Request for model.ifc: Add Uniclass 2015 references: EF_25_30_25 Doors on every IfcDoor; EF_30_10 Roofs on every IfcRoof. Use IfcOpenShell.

First a look at what the model holds.

```python
import ifcopenshell

model = ifcopenshell.open("model.ifc")
print(model.schema)
print("classifications:", [c.Name for c in model.by_type("IfcClassification")])
for ifc_class in ("IfcDoor", "IfcRoof", "IfcStair", "IfcWall", "IfcWindow"):
    print(ifc_class, len(model.by_type(ifc_class)))
```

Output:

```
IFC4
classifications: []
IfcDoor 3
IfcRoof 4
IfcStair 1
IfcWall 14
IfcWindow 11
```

```python
import ifcopenshell
import ifcopenshell.api.classification

model = ifcopenshell.open("model.ifc")

system = ifcopenshell.api.classification.add_classification(model, classification="Uniclass 2015")

codes = {
    "IfcDoor": ("EF_25_30_25", "Doors"),
    "IfcRoof": ("EF_30_10", "Roofs"),
}
for ifc_class, (code, name) in codes.items():
    products = model.by_type(ifc_class)
    ifcopenshell.api.classification.add_reference(
        model, products=products, classification=system, identification=code, name=name
    )
    print(code, len(products))

model.write("model-out.ifc")
```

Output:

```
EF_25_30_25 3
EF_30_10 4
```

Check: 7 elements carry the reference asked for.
